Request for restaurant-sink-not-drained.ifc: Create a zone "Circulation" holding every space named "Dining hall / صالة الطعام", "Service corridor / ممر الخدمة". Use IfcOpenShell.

First a look at what the model holds.

```python
import ifcopenshell

model = ifcopenshell.open("restaurant-sink-not-drained.ifc")
print(model.schema)
seen = {}
for space in model.by_type("IfcSpace"):
    seen[space.LongName] = seen.get(space.LongName, 0) + 1
for name, count in sorted(seen.items(), key=str):
    print(count, "x", name)
print("zones:", [z.Name for z in model.by_type("IfcZone")][:20])
```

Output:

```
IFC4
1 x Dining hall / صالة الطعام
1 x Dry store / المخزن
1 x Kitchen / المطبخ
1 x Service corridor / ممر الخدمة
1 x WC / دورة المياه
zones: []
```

```python
import ifcopenshell
import ifcopenshell.api.group
import ifcopenshell.api.root

model = ifcopenshell.open("restaurant-sink-not-drained.ifc")

names = {"Dining hall / صالة الطعام", "Service corridor / ممر الخدمة"}
spaces = [s for s in model.by_type("IfcSpace") if s.LongName in names]

zone = ifcopenshell.api.root.create_entity(model, ifc_class="IfcZone", name="Circulation")
ifcopenshell.api.group.assign_group(model, products=spaces, group=zone)
print(len(spaces), "spaces in", zone.Name)

model.write("restaurant-sink-not-drained_rev.ifc")
```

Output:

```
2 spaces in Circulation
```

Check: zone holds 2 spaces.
